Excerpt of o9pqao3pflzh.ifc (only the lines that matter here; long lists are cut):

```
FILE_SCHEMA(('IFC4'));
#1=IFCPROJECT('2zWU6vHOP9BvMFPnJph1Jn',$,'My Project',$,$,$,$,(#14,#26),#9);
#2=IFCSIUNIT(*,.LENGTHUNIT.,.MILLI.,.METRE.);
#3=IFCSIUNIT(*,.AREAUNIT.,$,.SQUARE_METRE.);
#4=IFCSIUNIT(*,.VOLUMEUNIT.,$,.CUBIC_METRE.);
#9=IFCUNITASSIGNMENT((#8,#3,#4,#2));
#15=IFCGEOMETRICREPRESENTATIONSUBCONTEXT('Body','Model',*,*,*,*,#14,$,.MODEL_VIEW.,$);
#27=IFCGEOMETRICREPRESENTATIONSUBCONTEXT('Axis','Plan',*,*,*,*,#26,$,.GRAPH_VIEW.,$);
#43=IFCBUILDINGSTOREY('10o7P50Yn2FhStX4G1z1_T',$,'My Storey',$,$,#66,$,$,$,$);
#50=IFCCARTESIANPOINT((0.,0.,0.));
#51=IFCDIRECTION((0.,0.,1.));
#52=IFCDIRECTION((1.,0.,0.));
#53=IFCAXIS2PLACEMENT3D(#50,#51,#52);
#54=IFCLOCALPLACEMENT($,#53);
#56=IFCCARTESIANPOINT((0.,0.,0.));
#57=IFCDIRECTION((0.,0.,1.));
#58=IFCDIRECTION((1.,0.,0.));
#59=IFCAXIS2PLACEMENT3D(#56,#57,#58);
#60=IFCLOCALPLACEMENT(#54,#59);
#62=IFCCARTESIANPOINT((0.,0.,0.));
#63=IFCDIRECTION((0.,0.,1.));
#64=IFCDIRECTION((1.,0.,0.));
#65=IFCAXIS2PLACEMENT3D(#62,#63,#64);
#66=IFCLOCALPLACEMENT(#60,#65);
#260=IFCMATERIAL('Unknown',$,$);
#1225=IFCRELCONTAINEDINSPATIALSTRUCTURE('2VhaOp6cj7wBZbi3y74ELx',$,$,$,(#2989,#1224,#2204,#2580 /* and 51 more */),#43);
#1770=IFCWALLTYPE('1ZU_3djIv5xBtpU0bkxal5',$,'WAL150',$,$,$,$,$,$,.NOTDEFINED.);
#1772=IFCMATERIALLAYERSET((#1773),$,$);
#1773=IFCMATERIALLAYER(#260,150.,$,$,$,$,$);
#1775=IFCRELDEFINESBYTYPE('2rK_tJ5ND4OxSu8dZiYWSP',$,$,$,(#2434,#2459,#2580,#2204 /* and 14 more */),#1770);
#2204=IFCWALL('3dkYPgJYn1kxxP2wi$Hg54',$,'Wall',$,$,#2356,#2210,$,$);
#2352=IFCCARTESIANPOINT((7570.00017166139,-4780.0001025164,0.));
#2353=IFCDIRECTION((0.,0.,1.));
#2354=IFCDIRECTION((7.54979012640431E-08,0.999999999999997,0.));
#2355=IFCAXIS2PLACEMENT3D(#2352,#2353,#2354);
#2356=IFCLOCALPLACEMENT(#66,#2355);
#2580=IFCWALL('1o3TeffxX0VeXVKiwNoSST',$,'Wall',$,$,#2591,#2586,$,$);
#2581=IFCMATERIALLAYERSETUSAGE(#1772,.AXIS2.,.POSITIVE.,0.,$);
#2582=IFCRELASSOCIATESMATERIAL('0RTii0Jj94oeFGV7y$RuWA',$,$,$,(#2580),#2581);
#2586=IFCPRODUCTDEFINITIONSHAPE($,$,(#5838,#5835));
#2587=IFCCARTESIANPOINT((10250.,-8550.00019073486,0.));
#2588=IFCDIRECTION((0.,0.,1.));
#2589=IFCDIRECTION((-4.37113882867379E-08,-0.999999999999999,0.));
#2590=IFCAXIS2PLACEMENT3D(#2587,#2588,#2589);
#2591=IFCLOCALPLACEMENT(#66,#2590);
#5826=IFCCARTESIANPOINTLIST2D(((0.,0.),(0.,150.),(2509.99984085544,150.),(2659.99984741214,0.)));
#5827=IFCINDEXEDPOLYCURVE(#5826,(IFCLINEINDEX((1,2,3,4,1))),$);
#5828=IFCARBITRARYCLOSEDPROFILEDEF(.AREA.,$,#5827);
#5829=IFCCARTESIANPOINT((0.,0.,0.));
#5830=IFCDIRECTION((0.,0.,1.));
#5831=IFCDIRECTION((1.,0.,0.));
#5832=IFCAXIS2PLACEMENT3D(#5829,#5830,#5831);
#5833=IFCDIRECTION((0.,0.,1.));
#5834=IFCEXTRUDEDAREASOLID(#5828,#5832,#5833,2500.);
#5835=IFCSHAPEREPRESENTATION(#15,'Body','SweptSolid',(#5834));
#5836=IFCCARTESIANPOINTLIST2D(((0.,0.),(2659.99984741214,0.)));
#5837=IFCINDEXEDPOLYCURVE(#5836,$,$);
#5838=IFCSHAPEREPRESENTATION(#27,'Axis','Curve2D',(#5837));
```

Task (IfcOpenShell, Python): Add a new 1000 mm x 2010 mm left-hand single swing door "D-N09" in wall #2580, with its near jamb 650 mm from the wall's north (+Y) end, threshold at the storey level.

```python
import numpy as np
import ifcopenshell
import ifcopenshell.api.feature
import ifcopenshell.api.geometry
import ifcopenshell.api.root
import ifcopenshell.api.spatial
import ifcopenshell.geom
import ifcopenshell.util.element
import ifcopenshell.util.placement
import ifcopenshell.util.representation
import ifcopenshell.util.shape
import ifcopenshell.util.unit

model = ifcopenshell.open("o9pqao3pflzh.ifc")
unit_scale = ifcopenshell.util.unit.calculate_unit_scale(model)
settings = ifcopenshell.geom.settings()


def volume(element):
    """Net volume in cubic metres, openings subtracted."""
    shape = ifcopenshell.geom.create_shape(settings, element)
    return ifcopenshell.util.shape.get_volume(shape.geometry)


wall = model.by_guid("1o3TeffxX0VeXVKiwNoSST")
storey = ifcopenshell.util.element.get_container(wall, ifc_class="IfcBuildingStorey")
context = ifcopenshell.util.representation.get_context(model, "Model", "Body", "MODEL_VIEW")
before = volume(wall)

width, height, from_end, sill = 1, 2.01, 0.65, 0.0  # metres

# The wall runs along its own X axis, and the end named is its -X end.
wall_shape = ifcopenshell.geom.create_shape(settings, wall)
x, y, z = ifcopenshell.util.shape.get_vertices(wall_shape.geometry).T
start = x.min() + from_end
face, thickness = float(y.min()), float(y.max() - y.min())
wall_matrix = ifcopenshell.util.placement.get_local_placement(wall.ObjectPlacement)
level = ifcopenshell.util.placement.get_local_placement(storey.ObjectPlacement)[2, 3]


def in_wall(x, y):
    """Placement at x, y metres in the wall's axes, at sill height."""
    matrix = wall_matrix.copy()
    matrix[:, 3] = wall_matrix @ np.array([x / unit_scale, y / unit_scale, 0.0, 1.0])
    matrix[2, 3] = level + sill / unit_scale
    return matrix


# Opening: a box that overshoots both wall faces by 50 mm.
opening = ifcopenshell.api.root.create_entity(model, ifc_class="IfcOpeningElement", predefined_type="OPENING")
box = ifcopenshell.api.geometry.add_wall_representation(
    model, context=context, length=width, height=height, thickness=thickness + 0.1
)
ifcopenshell.api.geometry.assign_representation(model, product=opening, representation=box)
ifcopenshell.api.geometry.edit_object_placement(model, product=opening, matrix=in_wall(start, face - 0.05), is_si=False)
ifcopenshell.api.feature.add_feature(model, feature=opening, element=wall)

door = ifcopenshell.api.root.create_entity(model, ifc_class="IfcDoor", name="D-N09", predefined_type="DOOR")
door.OverallWidth, door.OverallHeight = width / unit_scale, height / unit_scale
door.OperationType = "SINGLE_SWING_LEFT"
body = ifcopenshell.api.geometry.add_door_representation(
    model,
    context=context,
    overall_width=door.OverallWidth,
    overall_height=door.OverallHeight,
    operation_type="SINGLE_SWING_LEFT",
    lining_properties={"LiningDepth": thickness / unit_scale, "ThresholdDepth": thickness / unit_scale},
)
ifcopenshell.api.geometry.assign_representation(model, product=door, representation=body)
ifcopenshell.api.spatial.assign_container(model, products=[door], relating_structure=storey)
ifcopenshell.api.feature.add_filling(model, opening=opening, element=door)

# The lining spans the wall, so the door starts at the wall face.
ifcopenshell.api.geometry.edit_object_placement(model, product=door, matrix=in_wall(start, face), is_si=False)

after = volume(wall)

print(f"wall volume {before:.3f} -> {after:.3f} m3")

model.write("o9pqao3pflzh_rev.ifc")
```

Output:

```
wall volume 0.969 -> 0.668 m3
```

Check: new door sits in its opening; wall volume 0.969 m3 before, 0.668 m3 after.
